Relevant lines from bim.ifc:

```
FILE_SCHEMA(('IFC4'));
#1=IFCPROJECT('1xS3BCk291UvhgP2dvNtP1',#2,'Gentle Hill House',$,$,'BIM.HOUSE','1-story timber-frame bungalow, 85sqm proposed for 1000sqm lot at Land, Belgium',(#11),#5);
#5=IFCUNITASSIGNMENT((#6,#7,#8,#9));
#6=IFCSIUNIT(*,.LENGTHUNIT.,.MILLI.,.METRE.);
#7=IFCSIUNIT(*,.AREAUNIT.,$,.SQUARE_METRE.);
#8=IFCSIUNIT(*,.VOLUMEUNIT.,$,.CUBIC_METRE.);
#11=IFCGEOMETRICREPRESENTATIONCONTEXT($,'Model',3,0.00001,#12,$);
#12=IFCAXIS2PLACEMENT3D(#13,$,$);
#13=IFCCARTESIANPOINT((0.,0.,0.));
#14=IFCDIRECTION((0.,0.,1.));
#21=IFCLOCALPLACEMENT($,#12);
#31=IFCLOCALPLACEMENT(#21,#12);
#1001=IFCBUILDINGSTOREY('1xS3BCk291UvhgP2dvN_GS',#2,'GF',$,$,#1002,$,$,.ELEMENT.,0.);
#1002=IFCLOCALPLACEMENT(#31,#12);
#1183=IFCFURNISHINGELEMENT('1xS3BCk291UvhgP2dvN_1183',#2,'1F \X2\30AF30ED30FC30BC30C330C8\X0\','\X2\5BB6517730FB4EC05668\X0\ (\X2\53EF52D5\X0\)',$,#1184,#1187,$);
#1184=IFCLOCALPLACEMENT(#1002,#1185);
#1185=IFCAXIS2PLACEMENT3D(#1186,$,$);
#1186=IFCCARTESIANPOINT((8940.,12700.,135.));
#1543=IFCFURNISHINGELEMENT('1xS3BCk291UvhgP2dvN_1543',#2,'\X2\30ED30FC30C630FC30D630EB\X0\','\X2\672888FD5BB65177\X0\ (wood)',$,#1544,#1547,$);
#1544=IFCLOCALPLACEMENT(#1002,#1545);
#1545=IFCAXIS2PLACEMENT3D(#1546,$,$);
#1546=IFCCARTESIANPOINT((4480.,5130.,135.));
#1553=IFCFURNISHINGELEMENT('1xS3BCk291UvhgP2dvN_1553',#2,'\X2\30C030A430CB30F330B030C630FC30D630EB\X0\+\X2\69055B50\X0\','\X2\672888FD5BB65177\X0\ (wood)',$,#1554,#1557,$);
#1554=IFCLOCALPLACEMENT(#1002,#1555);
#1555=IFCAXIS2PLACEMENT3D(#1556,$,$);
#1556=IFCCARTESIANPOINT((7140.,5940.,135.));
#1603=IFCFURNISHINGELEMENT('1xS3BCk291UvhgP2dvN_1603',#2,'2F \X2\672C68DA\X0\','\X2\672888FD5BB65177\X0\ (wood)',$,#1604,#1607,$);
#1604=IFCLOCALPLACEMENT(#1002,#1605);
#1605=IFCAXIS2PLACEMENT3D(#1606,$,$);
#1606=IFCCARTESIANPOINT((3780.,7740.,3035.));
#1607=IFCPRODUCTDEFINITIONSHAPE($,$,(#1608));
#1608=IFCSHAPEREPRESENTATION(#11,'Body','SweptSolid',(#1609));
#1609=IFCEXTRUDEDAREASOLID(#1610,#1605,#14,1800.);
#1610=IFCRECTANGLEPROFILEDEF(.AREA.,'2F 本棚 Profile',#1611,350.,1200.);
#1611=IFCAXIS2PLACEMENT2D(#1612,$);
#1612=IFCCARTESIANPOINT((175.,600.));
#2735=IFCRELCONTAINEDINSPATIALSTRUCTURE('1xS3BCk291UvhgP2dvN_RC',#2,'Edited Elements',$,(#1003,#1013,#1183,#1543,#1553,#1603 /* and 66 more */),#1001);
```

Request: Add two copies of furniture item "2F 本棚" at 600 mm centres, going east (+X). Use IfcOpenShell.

```python
import numpy as np
import ifcopenshell
import ifcopenshell.api.geometry
import ifcopenshell.api.root
import ifcopenshell.util.element
import ifcopenshell.util.placement
import ifcopenshell.util.unit

model = ifcopenshell.open("bim.ifc")
unit_scale = ifcopenshell.util.unit.calculate_unit_scale(model)


def reuse_history(source, copy):
    """copy_class also copies each property set's owner history, people and application; keep the originals."""
    for rel in copy.IsDefinedBy:
        if rel.is_a("IfcRelDefinesByProperties") and (history := rel.RelatingPropertyDefinition.OwnerHistory):
            rel.RelatingPropertyDefinition.OwnerHistory = source.OwnerHistory
            ifcopenshell.util.element.remove_deep2(model, history)


source = model.by_id(1603)
base = ifcopenshell.util.placement.get_local_placement(source.ObjectPlacement)
step = np.array([1.0, 0.0, 0.0]) * 0.6 / unit_scale

for i in range(1, 3):
    copy = ifcopenshell.api.root.copy_class(model, product=source)
    copy.Representation = ifcopenshell.util.element.copy_deep(
        model, source.Representation, exclude=["IfcGeometricRepresentationContext", "IfcRepresentationMap"]
    )
    reuse_history(source, copy)
    matrix = base.copy()
    matrix[:3, 3] += i * step
    print("added at", matrix[:3, 3].round(3) + 0.0)
    ifcopenshell.api.geometry.edit_object_placement(model, product=copy, matrix=matrix, is_si=False)

model.write("bim_updated.ifc")
```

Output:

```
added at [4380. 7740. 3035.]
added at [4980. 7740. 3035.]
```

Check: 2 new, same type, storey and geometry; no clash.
